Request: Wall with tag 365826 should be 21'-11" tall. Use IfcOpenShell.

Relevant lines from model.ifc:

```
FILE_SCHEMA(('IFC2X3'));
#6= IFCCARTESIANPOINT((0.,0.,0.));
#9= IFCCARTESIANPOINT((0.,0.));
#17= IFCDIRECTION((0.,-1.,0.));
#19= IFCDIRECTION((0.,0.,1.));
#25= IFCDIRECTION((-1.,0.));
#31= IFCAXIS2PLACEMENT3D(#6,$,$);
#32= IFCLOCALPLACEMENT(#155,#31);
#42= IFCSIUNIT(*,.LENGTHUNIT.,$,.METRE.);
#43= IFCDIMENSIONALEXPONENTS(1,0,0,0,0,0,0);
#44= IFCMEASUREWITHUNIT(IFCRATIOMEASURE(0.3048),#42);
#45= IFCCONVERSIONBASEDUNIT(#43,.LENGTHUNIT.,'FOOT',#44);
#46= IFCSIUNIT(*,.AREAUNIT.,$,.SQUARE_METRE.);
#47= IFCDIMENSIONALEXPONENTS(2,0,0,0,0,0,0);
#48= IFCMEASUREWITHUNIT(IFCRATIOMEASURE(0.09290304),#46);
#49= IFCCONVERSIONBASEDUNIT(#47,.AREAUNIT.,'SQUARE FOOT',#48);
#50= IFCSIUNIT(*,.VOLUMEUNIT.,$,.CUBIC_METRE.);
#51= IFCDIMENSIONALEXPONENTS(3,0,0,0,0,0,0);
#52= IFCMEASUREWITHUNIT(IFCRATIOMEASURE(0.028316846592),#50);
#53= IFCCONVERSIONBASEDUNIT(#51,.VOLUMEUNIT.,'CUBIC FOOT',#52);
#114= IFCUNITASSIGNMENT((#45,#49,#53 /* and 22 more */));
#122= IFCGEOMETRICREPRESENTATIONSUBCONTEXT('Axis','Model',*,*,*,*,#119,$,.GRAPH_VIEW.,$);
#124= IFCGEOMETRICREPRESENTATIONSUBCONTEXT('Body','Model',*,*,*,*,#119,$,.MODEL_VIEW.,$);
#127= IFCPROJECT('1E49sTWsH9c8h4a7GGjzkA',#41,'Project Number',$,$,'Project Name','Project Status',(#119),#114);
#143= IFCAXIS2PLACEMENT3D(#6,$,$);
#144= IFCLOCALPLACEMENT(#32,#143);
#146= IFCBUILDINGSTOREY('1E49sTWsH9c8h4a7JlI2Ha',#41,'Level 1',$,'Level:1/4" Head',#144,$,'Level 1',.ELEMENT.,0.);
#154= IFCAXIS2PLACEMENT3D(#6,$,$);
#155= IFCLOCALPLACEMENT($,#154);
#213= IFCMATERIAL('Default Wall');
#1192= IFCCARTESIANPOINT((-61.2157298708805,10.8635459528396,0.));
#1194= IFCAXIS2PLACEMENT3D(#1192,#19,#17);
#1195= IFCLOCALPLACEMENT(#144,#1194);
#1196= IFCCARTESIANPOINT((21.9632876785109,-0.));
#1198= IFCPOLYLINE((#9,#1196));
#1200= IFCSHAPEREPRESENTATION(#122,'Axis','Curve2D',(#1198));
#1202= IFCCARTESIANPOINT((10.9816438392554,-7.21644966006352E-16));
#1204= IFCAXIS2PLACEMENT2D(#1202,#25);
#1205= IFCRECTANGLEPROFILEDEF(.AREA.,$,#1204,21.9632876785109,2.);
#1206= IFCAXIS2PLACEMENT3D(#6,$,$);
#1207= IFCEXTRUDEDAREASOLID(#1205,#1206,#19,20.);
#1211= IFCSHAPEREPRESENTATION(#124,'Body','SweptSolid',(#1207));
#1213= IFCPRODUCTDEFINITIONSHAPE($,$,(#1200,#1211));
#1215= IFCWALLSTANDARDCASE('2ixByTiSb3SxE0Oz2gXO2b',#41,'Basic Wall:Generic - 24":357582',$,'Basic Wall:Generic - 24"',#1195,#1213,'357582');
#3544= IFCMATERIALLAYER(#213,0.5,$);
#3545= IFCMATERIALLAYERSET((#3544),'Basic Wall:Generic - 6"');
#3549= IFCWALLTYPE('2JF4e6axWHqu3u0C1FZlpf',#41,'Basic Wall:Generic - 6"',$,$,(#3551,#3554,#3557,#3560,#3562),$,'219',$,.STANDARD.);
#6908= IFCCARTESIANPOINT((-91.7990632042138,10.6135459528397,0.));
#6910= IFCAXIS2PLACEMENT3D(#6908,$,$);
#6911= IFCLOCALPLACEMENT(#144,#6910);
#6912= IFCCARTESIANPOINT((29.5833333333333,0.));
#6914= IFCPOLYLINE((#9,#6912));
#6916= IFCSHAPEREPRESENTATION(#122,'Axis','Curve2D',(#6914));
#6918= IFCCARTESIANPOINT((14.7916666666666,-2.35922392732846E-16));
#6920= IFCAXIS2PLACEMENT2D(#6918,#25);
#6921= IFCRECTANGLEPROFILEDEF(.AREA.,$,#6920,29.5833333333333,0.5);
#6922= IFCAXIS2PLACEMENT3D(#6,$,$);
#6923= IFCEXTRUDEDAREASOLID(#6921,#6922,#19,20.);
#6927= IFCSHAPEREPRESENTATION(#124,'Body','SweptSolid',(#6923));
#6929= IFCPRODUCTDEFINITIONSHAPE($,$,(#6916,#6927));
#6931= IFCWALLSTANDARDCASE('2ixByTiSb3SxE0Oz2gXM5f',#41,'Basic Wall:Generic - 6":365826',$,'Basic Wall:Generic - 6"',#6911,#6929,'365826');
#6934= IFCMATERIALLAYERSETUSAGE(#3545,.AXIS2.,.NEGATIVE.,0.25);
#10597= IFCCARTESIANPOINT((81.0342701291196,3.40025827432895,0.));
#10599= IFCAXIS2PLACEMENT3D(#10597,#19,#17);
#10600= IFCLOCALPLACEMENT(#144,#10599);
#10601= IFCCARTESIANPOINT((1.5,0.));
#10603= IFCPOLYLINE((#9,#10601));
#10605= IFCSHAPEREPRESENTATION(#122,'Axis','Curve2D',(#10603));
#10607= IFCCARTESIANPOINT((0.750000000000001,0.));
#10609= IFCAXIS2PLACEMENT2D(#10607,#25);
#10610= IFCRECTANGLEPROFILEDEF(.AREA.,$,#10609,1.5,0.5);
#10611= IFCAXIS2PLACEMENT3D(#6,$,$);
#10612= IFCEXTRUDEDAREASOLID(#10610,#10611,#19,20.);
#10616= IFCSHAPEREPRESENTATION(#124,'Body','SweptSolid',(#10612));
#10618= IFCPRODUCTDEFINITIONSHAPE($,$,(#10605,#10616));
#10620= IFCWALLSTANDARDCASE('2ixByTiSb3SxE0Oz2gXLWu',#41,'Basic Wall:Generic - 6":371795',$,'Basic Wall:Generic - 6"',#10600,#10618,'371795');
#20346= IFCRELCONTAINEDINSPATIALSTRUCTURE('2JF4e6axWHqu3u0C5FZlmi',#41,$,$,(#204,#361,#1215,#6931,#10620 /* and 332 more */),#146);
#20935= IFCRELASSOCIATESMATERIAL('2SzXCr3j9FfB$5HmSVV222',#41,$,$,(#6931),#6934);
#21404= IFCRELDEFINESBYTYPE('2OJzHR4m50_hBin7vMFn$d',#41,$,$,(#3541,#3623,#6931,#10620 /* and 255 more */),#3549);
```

```python
import ifcopenshell
import ifcopenshell.geom
import ifcopenshell.util.representation
import ifcopenshell.util.shape
import ifcopenshell.util.unit

model = ifcopenshell.open("model.ifc")
unit_scale = ifcopenshell.util.unit.calculate_unit_scale(model)
settings = ifcopenshell.geom.settings()


def volume(element):
    """Net volume in cubic metres, openings subtracted."""
    shape = ifcopenshell.geom.create_shape(settings, element)
    return ifcopenshell.util.shape.get_volume(shape.geometry)


wall = model.by_id(6931)
before = volume(wall)

body = ifcopenshell.util.representation.get_representation(wall, "Model", "Body")
solid = body.Items[0]
old_height = solid.Depth
solid.Depth = 263 * 0.0254 / unit_scale
after = volume(wall)

print(f"height {old_height:g} -> {solid.Depth:g}, volume {before:.3f} -> {after:.3f} m3")

model.write("model_updated.ifc")
```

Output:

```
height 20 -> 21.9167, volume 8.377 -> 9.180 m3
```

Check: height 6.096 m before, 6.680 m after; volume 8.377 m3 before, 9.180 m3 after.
